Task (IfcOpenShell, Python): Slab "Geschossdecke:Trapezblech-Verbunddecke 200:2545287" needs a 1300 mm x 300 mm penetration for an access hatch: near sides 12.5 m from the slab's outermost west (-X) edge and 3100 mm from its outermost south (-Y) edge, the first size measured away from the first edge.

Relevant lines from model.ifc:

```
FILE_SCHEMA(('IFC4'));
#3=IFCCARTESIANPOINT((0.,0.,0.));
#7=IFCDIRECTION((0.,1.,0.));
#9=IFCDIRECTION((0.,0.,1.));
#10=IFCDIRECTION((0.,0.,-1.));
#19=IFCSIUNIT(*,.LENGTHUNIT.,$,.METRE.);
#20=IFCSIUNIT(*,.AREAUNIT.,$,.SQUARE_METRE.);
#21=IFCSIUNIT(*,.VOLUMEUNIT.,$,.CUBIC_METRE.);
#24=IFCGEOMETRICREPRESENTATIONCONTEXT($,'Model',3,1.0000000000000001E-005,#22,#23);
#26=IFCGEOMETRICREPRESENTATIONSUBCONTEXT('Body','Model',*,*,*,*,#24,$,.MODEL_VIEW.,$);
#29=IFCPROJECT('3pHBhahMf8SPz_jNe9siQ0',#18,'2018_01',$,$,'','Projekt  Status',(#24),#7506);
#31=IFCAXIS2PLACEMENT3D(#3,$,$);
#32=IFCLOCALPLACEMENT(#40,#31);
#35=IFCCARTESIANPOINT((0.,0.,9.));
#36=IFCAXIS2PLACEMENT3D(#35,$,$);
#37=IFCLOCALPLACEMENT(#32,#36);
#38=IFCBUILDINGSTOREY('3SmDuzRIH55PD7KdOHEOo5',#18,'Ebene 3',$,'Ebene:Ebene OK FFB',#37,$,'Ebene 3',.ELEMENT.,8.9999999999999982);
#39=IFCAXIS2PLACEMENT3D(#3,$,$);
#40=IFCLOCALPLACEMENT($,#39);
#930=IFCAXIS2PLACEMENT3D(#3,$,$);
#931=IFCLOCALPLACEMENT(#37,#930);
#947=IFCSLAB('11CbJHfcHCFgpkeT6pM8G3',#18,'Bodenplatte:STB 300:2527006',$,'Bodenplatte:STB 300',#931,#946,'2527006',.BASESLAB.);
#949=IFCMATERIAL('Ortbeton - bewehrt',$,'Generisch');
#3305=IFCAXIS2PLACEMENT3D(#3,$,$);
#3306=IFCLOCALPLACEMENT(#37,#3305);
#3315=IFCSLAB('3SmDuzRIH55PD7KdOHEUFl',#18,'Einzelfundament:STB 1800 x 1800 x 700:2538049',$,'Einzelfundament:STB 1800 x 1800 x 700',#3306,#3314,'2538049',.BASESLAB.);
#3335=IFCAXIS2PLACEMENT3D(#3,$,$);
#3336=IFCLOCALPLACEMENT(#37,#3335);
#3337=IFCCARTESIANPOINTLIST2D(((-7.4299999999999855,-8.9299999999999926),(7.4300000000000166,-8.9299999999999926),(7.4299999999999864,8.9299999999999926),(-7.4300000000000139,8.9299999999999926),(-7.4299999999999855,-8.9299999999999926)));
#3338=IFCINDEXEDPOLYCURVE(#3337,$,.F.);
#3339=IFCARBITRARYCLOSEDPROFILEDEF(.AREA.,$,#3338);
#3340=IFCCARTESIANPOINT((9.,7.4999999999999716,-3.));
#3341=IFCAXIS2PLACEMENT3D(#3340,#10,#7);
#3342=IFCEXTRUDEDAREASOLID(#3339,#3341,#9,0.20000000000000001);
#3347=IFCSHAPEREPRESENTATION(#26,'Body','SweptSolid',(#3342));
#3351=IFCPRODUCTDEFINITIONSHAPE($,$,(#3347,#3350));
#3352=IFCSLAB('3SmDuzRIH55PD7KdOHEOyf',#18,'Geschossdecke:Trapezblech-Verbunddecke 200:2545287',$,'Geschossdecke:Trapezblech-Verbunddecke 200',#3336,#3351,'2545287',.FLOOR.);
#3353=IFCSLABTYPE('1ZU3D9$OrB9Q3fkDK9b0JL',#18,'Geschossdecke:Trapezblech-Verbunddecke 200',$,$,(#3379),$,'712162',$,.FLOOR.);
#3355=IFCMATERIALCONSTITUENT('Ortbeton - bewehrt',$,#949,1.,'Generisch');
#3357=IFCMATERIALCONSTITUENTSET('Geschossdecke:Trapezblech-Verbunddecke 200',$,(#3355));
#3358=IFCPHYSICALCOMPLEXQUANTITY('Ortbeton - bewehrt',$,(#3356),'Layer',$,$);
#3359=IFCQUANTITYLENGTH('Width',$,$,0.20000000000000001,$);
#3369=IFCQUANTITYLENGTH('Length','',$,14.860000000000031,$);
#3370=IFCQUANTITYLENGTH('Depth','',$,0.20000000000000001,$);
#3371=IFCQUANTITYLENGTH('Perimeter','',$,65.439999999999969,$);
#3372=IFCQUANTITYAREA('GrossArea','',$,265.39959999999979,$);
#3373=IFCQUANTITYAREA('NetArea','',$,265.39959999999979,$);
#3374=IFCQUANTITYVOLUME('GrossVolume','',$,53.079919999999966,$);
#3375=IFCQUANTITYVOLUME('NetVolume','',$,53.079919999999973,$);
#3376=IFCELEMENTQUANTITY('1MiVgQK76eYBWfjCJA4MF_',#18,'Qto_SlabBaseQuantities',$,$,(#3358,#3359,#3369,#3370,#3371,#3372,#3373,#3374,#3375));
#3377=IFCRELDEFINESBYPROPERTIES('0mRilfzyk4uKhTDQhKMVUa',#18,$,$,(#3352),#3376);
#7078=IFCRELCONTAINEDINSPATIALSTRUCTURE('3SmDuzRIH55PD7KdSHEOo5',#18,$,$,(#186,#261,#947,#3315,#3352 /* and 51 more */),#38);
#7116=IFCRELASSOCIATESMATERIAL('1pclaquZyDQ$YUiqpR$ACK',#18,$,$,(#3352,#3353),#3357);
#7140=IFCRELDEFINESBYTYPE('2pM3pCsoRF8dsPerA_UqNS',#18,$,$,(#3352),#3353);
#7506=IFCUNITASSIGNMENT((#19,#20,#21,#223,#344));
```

```python
import numpy as np
import ifcopenshell
import ifcopenshell.api.feature
import ifcopenshell.api.geometry
import ifcopenshell.api.pset
import ifcopenshell.api.root
import ifcopenshell.geom
import ifcopenshell.util.element
import ifcopenshell.util.placement
import ifcopenshell.util.representation
import ifcopenshell.util.shape
import ifcopenshell.util.unit

model = ifcopenshell.open("model.ifc")
unit_scale = ifcopenshell.util.unit.calculate_unit_scale(model)
area_scale = ifcopenshell.util.unit.calculate_unit_scale(model, "AREAUNIT")
volume_scale = ifcopenshell.util.unit.calculate_unit_scale(model, "VOLUMEUNIT")
settings = ifcopenshell.geom.settings()


def volume(element):
    """Net volume in cubic metres, openings subtracted."""
    shape = ifcopenshell.geom.create_shape(settings, element)
    return ifcopenshell.util.shape.get_volume(shape.geometry)


slab = model.by_guid("3SmDuzRIH55PD7KdOHEOyf")
before = volume(slab)

# Extent in the slab's own axes, in metres. The edges named are its -X and -Y sides.
slab_shape = ifcopenshell.geom.create_shape(settings, slab)
vertices = ifcopenshell.util.shape.get_vertices(slab_shape.geometry)
x_min, y_min, bottom = vertices.min(axis=0)
top = vertices[:, 2].max()

opening = ifcopenshell.api.root.create_entity(model, ifc_class="IfcOpeningElement", name="Access hatch opening", predefined_type="OPENING")
context = ifcopenshell.util.representation.get_context(model, "Model", "Body", "MODEL_VIEW")
width, depth = 1.3, 0.3
outline = [(0.0, 0.0), (width, 0.0), (width, depth), (0.0, depth), (0.0, 0.0)]
# Overshoot both faces by 50 mm so the cut is clean.
shape = ifcopenshell.api.geometry.add_slab_representation(
    model, context=context, depth=top - bottom + 0.1, polyline=outline
)
ifcopenshell.api.geometry.assign_representation(model, product=opening, representation=shape)

matrix = ifcopenshell.util.placement.get_local_placement(slab.ObjectPlacement)
matrix[:, 3] = matrix @ np.append(np.array([x_min + 12.5, y_min + 3.1, bottom - 0.05]) / unit_scale, 1.0)
ifcopenshell.api.geometry.edit_object_placement(model, product=opening, matrix=matrix, is_si=False)
ifcopenshell.api.feature.add_feature(model, feature=opening, element=slab)

after = volume(slab)

# Update the slab's stored quantities.
qto = model.by_id(ifcopenshell.util.element.get_pset(slab, "Qto_SlabBaseQuantities", should_inherit=False)["id"])
ifcopenshell.api.pset.edit_qto(model, qto=qto, properties={
    "NetArea": after / (top - bottom) / area_scale,
    "NetVolume": after / volume_scale,
})

print(f"slab volume {before:.3f} -> {after:.3f} m3")

model.write("model_v2.ifc")
```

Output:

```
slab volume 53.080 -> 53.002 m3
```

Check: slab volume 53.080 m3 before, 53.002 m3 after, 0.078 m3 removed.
